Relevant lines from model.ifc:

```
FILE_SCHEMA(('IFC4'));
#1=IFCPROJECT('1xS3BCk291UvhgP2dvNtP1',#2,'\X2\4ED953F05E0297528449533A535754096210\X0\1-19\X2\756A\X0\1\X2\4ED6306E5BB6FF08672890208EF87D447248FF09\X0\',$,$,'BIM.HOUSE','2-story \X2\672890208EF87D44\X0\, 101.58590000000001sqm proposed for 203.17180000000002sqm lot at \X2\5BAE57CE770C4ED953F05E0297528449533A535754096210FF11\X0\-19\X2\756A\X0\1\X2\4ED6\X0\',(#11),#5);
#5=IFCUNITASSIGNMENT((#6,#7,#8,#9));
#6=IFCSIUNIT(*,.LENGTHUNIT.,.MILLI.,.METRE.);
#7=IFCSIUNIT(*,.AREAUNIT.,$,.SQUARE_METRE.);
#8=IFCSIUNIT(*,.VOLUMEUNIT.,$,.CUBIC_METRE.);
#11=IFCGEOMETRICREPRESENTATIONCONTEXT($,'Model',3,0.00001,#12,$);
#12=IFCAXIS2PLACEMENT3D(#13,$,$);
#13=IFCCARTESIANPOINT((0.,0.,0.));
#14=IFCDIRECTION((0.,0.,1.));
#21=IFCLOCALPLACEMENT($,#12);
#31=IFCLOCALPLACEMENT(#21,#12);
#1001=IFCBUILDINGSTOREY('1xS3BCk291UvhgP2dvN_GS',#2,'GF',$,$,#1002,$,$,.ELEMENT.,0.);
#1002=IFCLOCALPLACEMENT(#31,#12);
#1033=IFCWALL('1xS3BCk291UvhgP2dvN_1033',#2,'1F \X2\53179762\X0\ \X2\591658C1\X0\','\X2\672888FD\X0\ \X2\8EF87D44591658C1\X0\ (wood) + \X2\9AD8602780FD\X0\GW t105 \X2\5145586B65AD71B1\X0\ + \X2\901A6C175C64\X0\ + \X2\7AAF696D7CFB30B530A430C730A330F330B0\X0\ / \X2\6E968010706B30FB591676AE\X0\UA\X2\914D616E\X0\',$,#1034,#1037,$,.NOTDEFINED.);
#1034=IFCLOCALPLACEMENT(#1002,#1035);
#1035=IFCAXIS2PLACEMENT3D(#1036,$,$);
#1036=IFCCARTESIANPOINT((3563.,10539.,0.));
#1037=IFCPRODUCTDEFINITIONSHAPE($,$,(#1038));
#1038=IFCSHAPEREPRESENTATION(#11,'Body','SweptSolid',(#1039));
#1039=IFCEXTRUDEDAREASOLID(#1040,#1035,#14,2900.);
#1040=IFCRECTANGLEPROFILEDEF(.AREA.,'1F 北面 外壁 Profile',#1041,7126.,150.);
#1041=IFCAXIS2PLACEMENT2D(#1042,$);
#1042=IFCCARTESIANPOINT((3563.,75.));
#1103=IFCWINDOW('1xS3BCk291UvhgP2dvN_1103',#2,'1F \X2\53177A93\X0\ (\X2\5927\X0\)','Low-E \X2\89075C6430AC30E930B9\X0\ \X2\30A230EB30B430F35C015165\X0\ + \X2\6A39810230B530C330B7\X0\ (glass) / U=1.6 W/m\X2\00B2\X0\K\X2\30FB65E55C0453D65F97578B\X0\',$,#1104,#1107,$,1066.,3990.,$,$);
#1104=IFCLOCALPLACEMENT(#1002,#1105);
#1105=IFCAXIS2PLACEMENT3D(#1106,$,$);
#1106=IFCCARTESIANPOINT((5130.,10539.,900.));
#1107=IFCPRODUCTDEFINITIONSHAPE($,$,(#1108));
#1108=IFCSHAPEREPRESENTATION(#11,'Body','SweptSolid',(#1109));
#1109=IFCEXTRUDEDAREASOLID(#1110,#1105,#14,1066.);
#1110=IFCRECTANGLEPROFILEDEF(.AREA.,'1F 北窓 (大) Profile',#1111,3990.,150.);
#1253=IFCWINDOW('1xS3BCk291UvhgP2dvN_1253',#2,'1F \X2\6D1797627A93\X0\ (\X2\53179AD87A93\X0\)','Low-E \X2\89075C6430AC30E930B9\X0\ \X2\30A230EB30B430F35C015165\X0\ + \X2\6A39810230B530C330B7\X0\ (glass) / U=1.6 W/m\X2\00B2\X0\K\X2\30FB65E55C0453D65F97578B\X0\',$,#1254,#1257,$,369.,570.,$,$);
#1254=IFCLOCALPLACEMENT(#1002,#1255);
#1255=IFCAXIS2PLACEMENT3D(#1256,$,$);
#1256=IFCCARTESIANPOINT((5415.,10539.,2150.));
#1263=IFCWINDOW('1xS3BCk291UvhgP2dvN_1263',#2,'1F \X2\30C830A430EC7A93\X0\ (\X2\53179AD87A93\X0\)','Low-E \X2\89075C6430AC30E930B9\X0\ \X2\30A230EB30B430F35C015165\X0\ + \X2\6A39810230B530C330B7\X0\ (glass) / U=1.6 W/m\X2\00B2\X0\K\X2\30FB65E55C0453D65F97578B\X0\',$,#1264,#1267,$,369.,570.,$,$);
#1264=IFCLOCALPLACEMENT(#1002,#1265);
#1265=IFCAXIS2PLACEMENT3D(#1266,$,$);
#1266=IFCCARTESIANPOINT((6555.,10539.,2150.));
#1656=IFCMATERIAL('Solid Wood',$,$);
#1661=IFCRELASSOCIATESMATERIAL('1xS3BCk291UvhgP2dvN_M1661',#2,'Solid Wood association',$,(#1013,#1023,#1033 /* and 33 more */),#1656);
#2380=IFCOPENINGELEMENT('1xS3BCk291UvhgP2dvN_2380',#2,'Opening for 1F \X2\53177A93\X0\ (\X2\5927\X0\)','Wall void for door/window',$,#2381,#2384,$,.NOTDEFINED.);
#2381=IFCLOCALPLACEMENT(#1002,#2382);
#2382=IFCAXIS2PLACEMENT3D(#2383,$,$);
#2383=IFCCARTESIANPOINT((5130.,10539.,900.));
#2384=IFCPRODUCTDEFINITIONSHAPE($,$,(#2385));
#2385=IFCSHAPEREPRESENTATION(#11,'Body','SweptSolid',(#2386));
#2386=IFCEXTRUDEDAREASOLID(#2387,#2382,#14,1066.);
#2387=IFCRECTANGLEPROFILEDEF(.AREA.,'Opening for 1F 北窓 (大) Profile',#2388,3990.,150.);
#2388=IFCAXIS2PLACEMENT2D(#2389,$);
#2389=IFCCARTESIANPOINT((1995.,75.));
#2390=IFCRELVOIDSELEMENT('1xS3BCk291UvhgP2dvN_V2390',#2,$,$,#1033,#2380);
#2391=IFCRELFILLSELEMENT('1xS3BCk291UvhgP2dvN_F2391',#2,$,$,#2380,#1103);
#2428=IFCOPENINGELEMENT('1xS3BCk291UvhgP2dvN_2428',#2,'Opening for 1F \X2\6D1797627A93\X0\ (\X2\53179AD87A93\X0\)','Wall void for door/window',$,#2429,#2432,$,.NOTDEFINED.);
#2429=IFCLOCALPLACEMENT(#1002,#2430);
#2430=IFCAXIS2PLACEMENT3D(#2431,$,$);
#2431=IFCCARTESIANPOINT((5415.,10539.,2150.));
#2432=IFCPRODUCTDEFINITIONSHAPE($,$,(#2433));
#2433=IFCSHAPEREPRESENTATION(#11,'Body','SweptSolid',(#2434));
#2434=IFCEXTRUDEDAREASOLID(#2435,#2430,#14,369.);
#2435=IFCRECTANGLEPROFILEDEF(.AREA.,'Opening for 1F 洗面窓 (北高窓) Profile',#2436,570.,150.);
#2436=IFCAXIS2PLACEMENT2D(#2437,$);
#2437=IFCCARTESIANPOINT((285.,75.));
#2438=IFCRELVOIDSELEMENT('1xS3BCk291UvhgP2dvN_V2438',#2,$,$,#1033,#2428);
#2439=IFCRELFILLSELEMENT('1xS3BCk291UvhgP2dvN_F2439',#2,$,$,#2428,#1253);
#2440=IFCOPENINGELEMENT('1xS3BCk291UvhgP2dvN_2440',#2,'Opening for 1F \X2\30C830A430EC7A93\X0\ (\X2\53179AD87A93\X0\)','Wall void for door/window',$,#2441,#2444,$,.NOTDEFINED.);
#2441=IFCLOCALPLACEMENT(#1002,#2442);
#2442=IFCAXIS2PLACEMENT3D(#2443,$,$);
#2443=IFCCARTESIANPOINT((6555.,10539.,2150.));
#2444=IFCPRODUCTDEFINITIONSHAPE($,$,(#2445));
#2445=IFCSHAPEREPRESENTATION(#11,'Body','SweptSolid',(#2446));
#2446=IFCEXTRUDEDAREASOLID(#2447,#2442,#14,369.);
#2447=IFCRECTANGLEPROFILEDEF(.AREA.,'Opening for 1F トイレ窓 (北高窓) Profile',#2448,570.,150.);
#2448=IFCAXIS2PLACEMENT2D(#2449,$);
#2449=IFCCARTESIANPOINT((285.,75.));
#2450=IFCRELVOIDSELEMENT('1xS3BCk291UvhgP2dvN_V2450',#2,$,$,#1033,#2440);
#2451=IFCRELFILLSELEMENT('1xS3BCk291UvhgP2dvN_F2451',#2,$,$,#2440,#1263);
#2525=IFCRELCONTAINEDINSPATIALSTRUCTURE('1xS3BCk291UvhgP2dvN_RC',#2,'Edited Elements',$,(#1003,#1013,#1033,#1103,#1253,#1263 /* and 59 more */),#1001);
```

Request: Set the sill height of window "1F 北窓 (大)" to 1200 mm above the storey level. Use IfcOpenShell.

```python
import numpy as np
import ifcopenshell
import ifcopenshell.api.geometry
import ifcopenshell.geom
import ifcopenshell.util.element
import ifcopenshell.util.placement
import ifcopenshell.util.shape
import ifcopenshell.util.unit

model = ifcopenshell.open("model.ifc")
unit_scale = ifcopenshell.util.unit.calculate_unit_scale(model)

window = model.by_guid("1xS3BCk291UvhgP2dvN_1103")
opening = window.FillsVoids[0].RelatingOpeningElement
storey = ifcopenshell.util.element.get_container(window, ifc_class="IfcBuildingStorey")
level = ifcopenshell.util.placement.get_local_placement(storey.ObjectPlacement)[2, 3]

# The opening's origin need not be at the sill, so measure its lowest point.
shape = ifcopenshell.geom.create_shape(ifcopenshell.geom.settings(), opening)
bottom = ifcopenshell.util.shape.get_shape_bottom_elevation(shape, shape.geometry) / unit_scale
dz = level + 1.2 / unit_scale - bottom

shift = np.array([0.0, 0.0, dz])
# The window is not placed relative to its opening, so move both.
for product in (opening, window):
    matrix = ifcopenshell.util.placement.get_local_placement(product.ObjectPlacement)
    matrix[:3, 3] += shift
    ifcopenshell.api.geometry.edit_object_placement(model, product=product, matrix=matrix, is_si=False)

print(f"moved by {dz * unit_scale:+.3f} m")

model.write("model_rev.ifc")
```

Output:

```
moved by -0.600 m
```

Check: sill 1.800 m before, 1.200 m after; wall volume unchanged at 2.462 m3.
